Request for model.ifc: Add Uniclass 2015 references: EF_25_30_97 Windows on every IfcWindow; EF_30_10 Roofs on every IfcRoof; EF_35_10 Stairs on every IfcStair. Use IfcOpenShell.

First a look at what the model holds.

```python
import ifcopenshell

model = ifcopenshell.open("model.ifc")
print(model.schema)
print("classifications:", [c.Name for c in model.by_type("IfcClassification")])
for ifc_class in ("IfcDoor", "IfcRoof", "IfcStair", "IfcWall", "IfcWindow"):
    print(ifc_class, len(model.by_type(ifc_class)))
```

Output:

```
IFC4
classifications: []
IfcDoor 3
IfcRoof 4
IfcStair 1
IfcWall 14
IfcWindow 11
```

```python
import ifcopenshell
import ifcopenshell.api.classification

model = ifcopenshell.open("model.ifc")

system = ifcopenshell.api.classification.add_classification(model, classification="Uniclass 2015")

codes = {
    "IfcWindow": ("EF_25_30_97", "Windows"),
    "IfcRoof": ("EF_30_10", "Roofs"),
    "IfcStair": ("EF_35_10", "Stairs"),
}
for ifc_class, (code, name) in codes.items():
    products = model.by_type(ifc_class)
    ifcopenshell.api.classification.add_reference(
        model, products=products, classification=system, identification=code, name=name
    )
    print(code, len(products))

model.write("model_rev.ifc")
```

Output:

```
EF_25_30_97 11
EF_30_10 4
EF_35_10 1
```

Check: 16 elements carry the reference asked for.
